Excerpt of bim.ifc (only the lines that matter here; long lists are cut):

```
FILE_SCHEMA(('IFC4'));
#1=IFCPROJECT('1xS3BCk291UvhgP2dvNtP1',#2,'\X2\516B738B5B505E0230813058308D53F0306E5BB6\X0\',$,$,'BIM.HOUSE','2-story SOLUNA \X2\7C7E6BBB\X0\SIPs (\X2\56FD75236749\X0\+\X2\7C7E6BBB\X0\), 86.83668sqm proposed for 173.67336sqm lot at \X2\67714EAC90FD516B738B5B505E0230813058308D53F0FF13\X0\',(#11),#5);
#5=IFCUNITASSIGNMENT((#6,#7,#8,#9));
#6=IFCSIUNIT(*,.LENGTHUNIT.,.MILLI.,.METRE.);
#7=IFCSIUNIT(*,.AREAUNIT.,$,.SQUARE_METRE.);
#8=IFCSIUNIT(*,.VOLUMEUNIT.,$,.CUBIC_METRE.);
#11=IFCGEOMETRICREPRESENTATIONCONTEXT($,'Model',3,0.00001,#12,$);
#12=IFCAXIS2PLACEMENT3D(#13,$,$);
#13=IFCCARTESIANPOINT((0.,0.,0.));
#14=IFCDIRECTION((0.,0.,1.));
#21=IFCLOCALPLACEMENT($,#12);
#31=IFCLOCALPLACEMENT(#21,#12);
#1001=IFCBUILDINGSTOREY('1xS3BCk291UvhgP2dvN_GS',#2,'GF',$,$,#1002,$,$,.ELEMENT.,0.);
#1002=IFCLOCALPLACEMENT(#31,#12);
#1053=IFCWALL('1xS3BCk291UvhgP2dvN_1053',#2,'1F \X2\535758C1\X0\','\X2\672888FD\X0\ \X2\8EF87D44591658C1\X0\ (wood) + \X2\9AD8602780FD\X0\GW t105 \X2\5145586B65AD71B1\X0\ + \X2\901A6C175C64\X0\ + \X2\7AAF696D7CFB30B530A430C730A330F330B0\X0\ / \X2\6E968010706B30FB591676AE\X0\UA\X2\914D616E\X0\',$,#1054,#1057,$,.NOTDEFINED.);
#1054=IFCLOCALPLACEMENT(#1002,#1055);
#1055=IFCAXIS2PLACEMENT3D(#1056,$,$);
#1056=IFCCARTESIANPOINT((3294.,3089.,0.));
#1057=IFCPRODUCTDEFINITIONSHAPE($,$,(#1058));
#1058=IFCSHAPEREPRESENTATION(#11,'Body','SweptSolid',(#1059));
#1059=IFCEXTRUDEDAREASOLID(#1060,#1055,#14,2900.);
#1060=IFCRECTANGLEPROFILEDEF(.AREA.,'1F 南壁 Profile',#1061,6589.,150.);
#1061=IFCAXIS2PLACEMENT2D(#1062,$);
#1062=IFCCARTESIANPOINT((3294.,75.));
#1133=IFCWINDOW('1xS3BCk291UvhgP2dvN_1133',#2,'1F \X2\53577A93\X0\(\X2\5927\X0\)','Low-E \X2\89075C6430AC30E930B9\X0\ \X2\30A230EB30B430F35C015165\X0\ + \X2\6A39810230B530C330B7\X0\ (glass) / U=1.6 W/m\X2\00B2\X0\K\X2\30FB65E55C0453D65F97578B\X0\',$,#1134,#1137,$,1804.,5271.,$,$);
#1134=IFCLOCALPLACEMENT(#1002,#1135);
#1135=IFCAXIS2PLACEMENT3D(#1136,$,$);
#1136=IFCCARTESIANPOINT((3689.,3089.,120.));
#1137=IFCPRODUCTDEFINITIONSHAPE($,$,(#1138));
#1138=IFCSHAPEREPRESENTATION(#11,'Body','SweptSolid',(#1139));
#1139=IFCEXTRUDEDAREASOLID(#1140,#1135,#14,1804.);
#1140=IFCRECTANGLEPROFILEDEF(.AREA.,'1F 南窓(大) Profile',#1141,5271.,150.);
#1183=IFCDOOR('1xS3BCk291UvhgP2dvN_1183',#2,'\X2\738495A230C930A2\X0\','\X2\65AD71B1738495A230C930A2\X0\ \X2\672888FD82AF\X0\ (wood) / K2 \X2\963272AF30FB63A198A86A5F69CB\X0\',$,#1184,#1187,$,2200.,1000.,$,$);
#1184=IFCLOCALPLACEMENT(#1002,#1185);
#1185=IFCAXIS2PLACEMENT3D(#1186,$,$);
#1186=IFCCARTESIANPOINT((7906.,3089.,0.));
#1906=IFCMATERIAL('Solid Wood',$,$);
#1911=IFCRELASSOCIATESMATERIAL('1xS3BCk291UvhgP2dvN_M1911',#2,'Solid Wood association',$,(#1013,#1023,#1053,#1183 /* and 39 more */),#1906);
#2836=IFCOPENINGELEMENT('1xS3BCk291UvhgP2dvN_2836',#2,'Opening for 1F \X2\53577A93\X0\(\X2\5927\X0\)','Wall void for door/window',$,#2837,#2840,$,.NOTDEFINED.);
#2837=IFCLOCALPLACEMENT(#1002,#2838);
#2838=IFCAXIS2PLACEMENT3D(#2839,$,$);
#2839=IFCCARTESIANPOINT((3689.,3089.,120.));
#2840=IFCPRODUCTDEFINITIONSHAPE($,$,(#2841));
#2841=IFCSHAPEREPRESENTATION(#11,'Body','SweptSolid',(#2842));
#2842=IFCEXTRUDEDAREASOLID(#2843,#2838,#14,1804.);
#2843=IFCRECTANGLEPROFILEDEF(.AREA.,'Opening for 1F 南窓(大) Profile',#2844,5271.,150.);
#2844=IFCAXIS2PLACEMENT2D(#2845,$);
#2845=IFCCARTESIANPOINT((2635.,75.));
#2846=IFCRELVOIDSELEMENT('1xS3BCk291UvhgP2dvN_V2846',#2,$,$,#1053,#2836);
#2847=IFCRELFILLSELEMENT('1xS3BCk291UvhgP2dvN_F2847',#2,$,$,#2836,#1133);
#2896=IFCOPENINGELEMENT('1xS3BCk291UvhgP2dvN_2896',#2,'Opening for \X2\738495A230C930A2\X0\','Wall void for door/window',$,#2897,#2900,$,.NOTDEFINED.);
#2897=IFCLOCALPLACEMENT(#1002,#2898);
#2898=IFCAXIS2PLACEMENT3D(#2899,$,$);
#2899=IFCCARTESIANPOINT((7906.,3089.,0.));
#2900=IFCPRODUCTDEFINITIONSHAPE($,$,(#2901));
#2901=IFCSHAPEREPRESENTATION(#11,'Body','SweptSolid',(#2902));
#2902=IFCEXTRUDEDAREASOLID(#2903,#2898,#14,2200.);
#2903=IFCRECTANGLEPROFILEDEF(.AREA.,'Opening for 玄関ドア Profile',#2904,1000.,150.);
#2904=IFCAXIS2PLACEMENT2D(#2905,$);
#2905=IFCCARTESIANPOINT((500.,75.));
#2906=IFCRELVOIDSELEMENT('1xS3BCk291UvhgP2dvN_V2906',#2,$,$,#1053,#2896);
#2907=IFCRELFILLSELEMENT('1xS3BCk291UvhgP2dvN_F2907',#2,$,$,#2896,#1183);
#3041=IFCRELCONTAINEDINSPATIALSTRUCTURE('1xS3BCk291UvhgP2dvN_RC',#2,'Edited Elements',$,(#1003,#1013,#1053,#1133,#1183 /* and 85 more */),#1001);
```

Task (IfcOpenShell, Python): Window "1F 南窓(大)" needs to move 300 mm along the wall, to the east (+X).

```python
import ifcopenshell
import ifcopenshell.api.geometry
import ifcopenshell.util.placement

model = ifcopenshell.open("bim.ifc")

window = model.by_guid("1xS3BCk291UvhgP2dvN_1133")
opening = window.FillsVoids[0].RelatingOpeningElement
wall = opening.VoidsElements[0].RelatingBuildingElement

wall_matrix = ifcopenshell.util.placement.get_local_placement(wall.ObjectPlacement)
shift = wall_matrix[:3, 0] * 300.0
before = ifcopenshell.util.placement.get_local_placement(window.ObjectPlacement)[:3, 3].copy()

# The window is not placed relative to its opening, so move both.
for product in (opening, window):
    matrix = ifcopenshell.util.placement.get_local_placement(product.ObjectPlacement)
    matrix[:3, 3] += shift
    ifcopenshell.api.geometry.edit_object_placement(model, product=product, matrix=matrix, is_si=False)

after = ifcopenshell.util.placement.get_local_placement(window.ObjectPlacement)[:3, 3]
print("window moved by", (after - before).round(3) + 0.0)

model.write("bim_updated.ifc")
```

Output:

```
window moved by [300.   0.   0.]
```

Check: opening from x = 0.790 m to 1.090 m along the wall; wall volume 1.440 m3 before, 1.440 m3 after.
